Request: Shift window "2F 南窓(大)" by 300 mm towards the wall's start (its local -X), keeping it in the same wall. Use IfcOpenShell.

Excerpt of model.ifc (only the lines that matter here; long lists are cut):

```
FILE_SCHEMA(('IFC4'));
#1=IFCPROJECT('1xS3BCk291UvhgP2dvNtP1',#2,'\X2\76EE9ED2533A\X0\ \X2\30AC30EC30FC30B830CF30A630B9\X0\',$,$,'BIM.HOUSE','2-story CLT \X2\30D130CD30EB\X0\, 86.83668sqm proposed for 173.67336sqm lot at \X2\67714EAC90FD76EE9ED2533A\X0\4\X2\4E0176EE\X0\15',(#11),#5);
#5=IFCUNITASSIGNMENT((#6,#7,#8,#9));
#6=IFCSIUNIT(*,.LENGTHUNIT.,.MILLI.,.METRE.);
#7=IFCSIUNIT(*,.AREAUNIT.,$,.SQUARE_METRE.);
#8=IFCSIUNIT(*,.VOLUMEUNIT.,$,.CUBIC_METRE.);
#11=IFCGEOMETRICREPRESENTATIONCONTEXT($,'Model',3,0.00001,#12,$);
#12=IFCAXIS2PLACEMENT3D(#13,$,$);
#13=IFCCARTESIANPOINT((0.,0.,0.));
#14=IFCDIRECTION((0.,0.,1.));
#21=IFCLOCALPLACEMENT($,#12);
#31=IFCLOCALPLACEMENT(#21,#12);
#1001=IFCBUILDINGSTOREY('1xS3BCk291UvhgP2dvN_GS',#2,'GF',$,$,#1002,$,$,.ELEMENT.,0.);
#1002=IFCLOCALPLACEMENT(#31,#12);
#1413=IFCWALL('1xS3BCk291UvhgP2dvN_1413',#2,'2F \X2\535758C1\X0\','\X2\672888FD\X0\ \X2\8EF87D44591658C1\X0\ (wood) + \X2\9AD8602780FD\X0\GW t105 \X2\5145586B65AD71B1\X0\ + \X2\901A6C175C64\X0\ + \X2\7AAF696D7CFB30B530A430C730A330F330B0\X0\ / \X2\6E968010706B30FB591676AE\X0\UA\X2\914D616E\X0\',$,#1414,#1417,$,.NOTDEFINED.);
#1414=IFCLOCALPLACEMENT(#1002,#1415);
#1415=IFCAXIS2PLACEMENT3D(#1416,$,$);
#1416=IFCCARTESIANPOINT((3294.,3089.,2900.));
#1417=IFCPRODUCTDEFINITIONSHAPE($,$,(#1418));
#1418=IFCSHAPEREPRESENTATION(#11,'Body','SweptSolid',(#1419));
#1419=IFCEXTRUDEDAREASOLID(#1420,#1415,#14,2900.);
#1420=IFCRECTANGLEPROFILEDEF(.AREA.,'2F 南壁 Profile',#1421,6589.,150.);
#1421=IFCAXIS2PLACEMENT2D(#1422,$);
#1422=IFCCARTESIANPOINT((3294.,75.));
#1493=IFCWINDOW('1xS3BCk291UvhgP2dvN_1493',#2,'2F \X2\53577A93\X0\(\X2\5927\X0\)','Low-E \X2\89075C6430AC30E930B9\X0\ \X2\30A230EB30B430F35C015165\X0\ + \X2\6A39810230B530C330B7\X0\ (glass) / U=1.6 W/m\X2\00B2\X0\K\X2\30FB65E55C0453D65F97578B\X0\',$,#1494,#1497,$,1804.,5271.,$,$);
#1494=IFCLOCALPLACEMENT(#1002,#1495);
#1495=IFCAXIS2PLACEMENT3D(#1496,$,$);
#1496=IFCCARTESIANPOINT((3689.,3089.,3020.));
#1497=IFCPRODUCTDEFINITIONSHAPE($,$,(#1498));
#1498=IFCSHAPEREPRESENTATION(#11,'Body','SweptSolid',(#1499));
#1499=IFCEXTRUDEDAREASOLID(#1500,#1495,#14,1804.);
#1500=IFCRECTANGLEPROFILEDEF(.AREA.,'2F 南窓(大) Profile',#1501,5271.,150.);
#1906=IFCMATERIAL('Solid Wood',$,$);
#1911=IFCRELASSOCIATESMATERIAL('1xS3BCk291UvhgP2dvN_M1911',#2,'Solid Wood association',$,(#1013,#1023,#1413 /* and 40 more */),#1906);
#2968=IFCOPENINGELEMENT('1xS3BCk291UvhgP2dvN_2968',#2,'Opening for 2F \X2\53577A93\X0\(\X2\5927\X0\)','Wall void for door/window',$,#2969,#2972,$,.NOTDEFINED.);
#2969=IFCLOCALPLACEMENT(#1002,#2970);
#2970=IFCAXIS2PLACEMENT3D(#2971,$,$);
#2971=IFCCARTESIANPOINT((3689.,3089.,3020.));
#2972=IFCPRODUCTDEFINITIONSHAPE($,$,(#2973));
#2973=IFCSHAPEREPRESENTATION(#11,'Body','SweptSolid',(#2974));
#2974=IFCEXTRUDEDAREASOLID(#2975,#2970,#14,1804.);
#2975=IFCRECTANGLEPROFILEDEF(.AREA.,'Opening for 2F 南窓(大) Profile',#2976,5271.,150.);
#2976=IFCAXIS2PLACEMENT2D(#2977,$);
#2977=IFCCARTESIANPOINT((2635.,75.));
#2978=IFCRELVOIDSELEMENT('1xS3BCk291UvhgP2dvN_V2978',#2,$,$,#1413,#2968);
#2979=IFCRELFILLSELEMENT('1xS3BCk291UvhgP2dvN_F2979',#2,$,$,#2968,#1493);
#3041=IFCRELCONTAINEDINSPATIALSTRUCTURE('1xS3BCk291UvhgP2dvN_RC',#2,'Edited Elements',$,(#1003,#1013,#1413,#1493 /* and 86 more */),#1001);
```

```python
import ifcopenshell
import ifcopenshell.api.geometry
import ifcopenshell.util.placement
import ifcopenshell.util.unit

model = ifcopenshell.open("model.ifc")
unit_scale = ifcopenshell.util.unit.calculate_unit_scale(model)

window = model.by_id(1493)
opening = window.FillsVoids[0].RelatingOpeningElement
wall = opening.VoidsElements[0].RelatingBuildingElement

wall_matrix = ifcopenshell.util.placement.get_local_placement(wall.ObjectPlacement)
shift = wall_matrix[:3, 0] * -0.3 / unit_scale
before = ifcopenshell.util.placement.get_local_placement(window.ObjectPlacement)[:3, 3].copy()

# The window is not placed relative to its opening, so move both.
for product in (opening, window):
    matrix = ifcopenshell.util.placement.get_local_placement(product.ObjectPlacement)
    matrix[:3, 3] += shift
    ifcopenshell.api.geometry.edit_object_placement(model, product=product, matrix=matrix, is_si=False)

after = ifcopenshell.util.placement.get_local_placement(window.ObjectPlacement)[:3, 3]
print("window moved by", (after - before).round(3) + 0.0)

model.write("model_rev.ifc")
```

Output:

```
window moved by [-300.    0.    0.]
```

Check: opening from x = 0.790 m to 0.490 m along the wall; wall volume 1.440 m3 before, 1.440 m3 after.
